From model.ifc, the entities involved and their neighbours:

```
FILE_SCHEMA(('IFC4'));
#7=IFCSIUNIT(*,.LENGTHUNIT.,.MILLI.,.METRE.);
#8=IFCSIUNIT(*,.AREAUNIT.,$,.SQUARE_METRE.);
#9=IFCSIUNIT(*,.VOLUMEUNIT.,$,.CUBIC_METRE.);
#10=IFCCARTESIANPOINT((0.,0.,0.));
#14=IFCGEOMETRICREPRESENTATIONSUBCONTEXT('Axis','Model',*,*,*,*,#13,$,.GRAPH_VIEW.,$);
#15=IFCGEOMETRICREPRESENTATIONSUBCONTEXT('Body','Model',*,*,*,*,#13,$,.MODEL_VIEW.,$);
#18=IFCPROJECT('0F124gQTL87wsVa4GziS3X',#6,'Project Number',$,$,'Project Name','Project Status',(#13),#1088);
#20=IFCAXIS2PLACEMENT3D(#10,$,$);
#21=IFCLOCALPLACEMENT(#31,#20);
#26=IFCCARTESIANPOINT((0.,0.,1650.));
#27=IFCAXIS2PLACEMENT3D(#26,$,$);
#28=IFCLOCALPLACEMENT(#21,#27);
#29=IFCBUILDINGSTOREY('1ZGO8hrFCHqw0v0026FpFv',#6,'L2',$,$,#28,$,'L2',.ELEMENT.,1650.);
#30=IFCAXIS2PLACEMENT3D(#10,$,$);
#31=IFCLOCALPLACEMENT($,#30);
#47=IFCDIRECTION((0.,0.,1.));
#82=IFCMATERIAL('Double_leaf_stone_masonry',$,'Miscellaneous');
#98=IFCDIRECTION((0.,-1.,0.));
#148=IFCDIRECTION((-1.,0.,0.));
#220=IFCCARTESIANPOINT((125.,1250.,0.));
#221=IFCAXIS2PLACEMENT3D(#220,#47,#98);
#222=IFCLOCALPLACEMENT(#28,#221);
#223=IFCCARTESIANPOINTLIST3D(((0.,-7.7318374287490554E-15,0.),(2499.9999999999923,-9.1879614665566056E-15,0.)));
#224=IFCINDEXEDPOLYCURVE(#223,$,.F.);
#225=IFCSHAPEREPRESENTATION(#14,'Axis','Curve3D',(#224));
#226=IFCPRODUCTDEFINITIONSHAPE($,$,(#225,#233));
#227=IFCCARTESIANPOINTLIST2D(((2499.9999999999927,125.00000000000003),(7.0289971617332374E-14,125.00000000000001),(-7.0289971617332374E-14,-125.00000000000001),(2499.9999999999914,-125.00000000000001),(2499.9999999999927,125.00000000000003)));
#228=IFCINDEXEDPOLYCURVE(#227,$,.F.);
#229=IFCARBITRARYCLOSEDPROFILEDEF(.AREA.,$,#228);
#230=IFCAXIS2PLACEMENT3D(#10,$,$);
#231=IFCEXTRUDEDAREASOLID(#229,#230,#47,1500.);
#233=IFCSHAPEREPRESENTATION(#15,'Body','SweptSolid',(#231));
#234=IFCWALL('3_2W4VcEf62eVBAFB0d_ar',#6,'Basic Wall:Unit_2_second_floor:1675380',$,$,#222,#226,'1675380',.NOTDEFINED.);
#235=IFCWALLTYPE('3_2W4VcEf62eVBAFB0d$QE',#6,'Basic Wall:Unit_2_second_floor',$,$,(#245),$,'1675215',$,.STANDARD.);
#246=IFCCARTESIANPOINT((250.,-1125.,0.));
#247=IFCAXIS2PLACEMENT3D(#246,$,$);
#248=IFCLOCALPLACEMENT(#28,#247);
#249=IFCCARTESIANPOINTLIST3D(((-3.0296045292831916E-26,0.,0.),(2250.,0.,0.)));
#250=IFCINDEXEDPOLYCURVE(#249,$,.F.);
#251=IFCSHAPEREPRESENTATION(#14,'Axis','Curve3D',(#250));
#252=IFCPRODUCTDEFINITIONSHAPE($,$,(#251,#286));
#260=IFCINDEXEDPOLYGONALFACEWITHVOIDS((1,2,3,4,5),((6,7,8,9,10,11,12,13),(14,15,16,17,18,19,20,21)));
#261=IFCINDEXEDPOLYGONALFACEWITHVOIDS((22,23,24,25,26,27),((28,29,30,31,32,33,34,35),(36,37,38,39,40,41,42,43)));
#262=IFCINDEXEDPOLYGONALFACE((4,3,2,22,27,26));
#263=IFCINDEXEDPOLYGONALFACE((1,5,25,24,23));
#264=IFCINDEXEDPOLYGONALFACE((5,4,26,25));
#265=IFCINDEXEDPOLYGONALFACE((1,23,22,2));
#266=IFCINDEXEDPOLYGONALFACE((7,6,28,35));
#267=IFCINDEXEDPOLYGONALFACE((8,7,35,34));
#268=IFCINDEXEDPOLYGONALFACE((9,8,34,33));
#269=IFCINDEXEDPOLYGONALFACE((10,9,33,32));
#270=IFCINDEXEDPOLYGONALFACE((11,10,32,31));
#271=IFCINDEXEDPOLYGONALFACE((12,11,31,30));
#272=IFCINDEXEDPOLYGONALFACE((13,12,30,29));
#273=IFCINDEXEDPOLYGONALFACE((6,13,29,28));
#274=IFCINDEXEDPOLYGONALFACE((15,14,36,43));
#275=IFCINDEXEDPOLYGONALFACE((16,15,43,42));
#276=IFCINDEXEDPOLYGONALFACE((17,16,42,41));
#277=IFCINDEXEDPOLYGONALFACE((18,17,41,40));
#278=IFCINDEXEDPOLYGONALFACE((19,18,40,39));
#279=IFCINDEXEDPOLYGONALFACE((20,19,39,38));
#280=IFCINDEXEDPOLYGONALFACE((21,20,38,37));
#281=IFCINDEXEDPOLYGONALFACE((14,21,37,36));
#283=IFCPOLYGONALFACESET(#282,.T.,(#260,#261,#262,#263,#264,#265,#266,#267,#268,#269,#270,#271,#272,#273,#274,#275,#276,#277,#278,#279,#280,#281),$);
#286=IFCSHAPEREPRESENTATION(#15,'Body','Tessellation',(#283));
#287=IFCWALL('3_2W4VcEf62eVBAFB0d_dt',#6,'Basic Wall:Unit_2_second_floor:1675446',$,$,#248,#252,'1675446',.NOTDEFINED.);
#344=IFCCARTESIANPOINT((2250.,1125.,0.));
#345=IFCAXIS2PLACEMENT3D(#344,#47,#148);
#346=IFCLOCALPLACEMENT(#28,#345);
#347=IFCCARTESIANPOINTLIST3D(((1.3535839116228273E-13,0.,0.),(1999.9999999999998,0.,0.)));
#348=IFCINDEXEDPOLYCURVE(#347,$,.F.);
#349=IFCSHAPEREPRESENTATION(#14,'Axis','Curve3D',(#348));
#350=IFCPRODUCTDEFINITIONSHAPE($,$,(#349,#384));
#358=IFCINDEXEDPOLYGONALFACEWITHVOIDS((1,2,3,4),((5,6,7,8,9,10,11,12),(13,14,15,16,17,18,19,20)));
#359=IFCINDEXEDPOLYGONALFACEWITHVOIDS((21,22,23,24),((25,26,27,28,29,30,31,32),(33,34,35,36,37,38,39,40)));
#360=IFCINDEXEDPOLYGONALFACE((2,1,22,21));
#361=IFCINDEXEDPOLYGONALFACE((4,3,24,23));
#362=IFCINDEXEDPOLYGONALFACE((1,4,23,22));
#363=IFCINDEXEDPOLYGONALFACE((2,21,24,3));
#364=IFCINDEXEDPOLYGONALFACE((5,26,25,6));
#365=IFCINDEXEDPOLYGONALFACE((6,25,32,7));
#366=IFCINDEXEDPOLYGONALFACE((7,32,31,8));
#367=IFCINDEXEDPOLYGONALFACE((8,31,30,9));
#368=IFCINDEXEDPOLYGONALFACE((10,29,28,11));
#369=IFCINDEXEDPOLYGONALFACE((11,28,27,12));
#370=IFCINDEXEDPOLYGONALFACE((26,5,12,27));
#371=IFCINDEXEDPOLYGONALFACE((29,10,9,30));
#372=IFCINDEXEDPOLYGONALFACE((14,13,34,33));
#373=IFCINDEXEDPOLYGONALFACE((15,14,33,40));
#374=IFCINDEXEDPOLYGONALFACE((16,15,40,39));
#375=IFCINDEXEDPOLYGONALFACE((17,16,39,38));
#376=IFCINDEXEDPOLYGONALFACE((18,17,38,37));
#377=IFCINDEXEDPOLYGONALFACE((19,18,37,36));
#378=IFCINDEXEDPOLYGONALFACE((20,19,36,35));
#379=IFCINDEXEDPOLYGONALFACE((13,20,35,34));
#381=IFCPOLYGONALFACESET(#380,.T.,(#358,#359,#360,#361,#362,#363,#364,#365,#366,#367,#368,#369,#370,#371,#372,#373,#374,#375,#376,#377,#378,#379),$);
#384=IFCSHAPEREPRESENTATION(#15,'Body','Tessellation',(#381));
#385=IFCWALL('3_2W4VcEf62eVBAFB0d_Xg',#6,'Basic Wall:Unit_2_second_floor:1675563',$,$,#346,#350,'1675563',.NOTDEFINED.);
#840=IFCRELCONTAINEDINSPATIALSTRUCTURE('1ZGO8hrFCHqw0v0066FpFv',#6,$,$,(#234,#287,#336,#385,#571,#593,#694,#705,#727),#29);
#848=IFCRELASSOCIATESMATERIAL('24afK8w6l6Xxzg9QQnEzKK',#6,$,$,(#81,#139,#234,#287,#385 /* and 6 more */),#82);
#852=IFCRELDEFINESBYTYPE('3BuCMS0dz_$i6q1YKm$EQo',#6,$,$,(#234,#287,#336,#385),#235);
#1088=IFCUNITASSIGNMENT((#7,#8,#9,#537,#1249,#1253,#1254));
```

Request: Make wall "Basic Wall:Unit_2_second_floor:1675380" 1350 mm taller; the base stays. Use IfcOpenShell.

```python
import ifcopenshell
import ifcopenshell.geom
import ifcopenshell.util.representation
import ifcopenshell.util.shape
import ifcopenshell.util.unit

model = ifcopenshell.open("model.ifc")
unit_scale = ifcopenshell.util.unit.calculate_unit_scale(model)
settings = ifcopenshell.geom.settings()


def volume(element):
    """Net volume in cubic metres, openings subtracted."""
    shape = ifcopenshell.geom.create_shape(settings, element)
    return ifcopenshell.util.shape.get_volume(shape.geometry)


wall = model.by_id(234)
before = volume(wall)

body = ifcopenshell.util.representation.get_representation(wall, "Model", "Body")
solid = body.Items[0]
old_height = solid.Depth
solid.Depth += 1.35 / unit_scale
after = volume(wall)

print(f"height {old_height:g} -> {solid.Depth:g}, volume {before:.3f} -> {after:.3f} m3")

model.write("model-out.ifc")
```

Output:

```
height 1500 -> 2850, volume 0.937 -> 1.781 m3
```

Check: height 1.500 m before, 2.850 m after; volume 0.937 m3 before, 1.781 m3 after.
